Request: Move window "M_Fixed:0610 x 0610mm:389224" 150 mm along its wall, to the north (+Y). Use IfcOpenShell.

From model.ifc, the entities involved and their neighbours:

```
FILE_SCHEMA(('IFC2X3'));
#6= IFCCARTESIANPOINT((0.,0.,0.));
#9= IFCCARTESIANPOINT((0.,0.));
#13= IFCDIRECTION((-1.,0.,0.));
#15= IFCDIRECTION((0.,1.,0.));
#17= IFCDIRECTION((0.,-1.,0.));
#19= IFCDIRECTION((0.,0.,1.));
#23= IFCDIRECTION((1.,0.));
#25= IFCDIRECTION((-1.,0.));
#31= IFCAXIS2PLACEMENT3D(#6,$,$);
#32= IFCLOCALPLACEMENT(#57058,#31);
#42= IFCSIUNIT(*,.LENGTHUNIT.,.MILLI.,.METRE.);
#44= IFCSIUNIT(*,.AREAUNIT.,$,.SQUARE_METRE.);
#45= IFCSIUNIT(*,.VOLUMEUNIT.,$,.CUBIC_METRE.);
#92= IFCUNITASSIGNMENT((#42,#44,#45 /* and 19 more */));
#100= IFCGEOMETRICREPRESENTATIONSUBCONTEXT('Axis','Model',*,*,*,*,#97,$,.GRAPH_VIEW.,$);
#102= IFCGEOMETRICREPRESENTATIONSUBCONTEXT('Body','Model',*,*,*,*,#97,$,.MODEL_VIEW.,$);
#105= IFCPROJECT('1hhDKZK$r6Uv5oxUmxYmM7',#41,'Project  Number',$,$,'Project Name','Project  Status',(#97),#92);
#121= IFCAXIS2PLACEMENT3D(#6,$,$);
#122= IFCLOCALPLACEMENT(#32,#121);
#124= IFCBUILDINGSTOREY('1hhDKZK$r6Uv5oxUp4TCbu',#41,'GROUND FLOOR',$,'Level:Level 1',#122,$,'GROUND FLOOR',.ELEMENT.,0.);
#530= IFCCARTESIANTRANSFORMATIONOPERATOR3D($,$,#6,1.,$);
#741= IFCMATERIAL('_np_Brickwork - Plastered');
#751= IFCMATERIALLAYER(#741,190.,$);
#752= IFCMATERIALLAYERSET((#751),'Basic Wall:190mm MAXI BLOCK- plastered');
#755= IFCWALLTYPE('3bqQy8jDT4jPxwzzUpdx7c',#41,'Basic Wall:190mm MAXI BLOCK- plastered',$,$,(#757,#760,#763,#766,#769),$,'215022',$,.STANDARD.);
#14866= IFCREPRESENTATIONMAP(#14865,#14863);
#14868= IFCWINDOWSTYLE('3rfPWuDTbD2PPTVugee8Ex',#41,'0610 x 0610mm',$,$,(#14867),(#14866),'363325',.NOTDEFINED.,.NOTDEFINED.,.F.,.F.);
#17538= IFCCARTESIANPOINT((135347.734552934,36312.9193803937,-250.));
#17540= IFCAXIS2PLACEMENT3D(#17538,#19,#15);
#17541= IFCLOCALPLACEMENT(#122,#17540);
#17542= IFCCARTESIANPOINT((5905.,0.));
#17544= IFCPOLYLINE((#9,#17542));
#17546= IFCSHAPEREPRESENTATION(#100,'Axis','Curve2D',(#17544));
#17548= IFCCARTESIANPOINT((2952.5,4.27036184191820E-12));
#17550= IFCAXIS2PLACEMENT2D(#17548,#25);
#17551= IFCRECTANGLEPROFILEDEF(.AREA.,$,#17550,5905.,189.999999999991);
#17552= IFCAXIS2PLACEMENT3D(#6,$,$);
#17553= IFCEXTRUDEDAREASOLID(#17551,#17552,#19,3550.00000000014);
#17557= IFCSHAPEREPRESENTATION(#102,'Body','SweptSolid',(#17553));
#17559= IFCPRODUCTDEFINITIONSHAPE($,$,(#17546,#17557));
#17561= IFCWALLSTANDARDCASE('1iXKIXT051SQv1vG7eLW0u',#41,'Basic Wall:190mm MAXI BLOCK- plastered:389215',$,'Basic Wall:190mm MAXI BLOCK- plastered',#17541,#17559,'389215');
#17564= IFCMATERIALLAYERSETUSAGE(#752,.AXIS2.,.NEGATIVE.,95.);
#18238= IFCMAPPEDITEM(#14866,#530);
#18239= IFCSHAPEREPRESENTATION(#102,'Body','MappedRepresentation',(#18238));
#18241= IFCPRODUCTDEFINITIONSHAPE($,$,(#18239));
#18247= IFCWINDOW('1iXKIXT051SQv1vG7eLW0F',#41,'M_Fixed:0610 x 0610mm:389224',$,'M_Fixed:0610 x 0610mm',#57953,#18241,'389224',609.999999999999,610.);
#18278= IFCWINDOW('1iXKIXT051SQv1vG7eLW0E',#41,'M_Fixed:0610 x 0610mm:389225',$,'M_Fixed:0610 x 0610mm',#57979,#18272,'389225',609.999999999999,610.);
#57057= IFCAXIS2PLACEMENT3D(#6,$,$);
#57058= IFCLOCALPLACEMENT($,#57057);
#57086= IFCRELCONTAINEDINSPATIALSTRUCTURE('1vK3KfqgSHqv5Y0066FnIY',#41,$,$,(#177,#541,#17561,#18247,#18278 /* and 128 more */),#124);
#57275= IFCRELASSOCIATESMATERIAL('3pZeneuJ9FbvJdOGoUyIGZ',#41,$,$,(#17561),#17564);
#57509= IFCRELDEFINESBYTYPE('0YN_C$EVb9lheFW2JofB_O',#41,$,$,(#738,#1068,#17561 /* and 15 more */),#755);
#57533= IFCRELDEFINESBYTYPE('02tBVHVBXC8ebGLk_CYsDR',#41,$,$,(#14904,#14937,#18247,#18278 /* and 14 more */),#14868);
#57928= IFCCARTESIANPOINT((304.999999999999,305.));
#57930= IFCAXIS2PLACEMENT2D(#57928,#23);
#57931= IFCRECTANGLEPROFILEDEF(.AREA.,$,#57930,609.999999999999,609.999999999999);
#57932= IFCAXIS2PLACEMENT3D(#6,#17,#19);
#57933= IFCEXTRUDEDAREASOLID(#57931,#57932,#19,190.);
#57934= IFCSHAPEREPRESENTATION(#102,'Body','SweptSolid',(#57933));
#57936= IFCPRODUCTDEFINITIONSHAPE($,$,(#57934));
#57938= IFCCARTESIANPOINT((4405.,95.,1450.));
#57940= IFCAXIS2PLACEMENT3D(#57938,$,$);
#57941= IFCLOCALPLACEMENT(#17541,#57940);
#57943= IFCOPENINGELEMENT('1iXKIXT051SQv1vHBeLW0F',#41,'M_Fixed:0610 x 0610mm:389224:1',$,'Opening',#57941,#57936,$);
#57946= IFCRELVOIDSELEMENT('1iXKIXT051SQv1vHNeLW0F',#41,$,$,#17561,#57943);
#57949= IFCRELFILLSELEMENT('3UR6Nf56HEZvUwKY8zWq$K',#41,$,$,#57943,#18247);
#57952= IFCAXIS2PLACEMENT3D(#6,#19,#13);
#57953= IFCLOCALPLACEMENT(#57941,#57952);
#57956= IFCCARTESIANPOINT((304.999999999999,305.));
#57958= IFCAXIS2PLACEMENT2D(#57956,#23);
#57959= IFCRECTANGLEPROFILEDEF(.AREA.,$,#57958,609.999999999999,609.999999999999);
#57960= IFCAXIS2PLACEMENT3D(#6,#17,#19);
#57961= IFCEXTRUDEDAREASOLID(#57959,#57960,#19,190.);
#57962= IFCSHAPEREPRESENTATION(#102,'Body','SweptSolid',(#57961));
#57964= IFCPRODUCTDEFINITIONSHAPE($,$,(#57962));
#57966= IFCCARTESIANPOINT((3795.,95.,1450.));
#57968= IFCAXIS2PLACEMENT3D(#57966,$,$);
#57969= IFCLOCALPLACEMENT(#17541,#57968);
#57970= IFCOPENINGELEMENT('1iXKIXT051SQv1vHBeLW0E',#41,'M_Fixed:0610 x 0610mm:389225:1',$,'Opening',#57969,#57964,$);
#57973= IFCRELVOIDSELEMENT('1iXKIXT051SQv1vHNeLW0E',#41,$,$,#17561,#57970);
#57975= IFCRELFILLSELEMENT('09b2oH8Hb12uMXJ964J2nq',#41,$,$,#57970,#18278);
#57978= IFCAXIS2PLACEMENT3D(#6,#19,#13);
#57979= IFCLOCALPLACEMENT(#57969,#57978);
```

```python
import ifcopenshell
import ifcopenshell.api.geometry
import ifcopenshell.util.placement

model = ifcopenshell.open("model.ifc")

window = model.by_guid("1iXKIXT051SQv1vG7eLW0F")
opening = window.FillsVoids[0].RelatingOpeningElement
wall = opening.VoidsElements[0].RelatingBuildingElement

wall_matrix = ifcopenshell.util.placement.get_local_placement(wall.ObjectPlacement)
shift = wall_matrix[:3, 0] * 150.0
before = ifcopenshell.util.placement.get_local_placement(window.ObjectPlacement)[:3, 3].copy()

# The window is placed relative to its opening, so it follows when the opening moves.
matrix = ifcopenshell.util.placement.get_local_placement(opening.ObjectPlacement)
matrix[:3, 3] += shift
ifcopenshell.api.geometry.edit_object_placement(
    model, product=opening, matrix=matrix, is_si=False, should_transform_children=True
)

after = ifcopenshell.util.placement.get_local_placement(window.ObjectPlacement)[:3, 3]
print("window moved by", (after - before).round(3) + 0.0)

model.write("model_updated.ifc")
```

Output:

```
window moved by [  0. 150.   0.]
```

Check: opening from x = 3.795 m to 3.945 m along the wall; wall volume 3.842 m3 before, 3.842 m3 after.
